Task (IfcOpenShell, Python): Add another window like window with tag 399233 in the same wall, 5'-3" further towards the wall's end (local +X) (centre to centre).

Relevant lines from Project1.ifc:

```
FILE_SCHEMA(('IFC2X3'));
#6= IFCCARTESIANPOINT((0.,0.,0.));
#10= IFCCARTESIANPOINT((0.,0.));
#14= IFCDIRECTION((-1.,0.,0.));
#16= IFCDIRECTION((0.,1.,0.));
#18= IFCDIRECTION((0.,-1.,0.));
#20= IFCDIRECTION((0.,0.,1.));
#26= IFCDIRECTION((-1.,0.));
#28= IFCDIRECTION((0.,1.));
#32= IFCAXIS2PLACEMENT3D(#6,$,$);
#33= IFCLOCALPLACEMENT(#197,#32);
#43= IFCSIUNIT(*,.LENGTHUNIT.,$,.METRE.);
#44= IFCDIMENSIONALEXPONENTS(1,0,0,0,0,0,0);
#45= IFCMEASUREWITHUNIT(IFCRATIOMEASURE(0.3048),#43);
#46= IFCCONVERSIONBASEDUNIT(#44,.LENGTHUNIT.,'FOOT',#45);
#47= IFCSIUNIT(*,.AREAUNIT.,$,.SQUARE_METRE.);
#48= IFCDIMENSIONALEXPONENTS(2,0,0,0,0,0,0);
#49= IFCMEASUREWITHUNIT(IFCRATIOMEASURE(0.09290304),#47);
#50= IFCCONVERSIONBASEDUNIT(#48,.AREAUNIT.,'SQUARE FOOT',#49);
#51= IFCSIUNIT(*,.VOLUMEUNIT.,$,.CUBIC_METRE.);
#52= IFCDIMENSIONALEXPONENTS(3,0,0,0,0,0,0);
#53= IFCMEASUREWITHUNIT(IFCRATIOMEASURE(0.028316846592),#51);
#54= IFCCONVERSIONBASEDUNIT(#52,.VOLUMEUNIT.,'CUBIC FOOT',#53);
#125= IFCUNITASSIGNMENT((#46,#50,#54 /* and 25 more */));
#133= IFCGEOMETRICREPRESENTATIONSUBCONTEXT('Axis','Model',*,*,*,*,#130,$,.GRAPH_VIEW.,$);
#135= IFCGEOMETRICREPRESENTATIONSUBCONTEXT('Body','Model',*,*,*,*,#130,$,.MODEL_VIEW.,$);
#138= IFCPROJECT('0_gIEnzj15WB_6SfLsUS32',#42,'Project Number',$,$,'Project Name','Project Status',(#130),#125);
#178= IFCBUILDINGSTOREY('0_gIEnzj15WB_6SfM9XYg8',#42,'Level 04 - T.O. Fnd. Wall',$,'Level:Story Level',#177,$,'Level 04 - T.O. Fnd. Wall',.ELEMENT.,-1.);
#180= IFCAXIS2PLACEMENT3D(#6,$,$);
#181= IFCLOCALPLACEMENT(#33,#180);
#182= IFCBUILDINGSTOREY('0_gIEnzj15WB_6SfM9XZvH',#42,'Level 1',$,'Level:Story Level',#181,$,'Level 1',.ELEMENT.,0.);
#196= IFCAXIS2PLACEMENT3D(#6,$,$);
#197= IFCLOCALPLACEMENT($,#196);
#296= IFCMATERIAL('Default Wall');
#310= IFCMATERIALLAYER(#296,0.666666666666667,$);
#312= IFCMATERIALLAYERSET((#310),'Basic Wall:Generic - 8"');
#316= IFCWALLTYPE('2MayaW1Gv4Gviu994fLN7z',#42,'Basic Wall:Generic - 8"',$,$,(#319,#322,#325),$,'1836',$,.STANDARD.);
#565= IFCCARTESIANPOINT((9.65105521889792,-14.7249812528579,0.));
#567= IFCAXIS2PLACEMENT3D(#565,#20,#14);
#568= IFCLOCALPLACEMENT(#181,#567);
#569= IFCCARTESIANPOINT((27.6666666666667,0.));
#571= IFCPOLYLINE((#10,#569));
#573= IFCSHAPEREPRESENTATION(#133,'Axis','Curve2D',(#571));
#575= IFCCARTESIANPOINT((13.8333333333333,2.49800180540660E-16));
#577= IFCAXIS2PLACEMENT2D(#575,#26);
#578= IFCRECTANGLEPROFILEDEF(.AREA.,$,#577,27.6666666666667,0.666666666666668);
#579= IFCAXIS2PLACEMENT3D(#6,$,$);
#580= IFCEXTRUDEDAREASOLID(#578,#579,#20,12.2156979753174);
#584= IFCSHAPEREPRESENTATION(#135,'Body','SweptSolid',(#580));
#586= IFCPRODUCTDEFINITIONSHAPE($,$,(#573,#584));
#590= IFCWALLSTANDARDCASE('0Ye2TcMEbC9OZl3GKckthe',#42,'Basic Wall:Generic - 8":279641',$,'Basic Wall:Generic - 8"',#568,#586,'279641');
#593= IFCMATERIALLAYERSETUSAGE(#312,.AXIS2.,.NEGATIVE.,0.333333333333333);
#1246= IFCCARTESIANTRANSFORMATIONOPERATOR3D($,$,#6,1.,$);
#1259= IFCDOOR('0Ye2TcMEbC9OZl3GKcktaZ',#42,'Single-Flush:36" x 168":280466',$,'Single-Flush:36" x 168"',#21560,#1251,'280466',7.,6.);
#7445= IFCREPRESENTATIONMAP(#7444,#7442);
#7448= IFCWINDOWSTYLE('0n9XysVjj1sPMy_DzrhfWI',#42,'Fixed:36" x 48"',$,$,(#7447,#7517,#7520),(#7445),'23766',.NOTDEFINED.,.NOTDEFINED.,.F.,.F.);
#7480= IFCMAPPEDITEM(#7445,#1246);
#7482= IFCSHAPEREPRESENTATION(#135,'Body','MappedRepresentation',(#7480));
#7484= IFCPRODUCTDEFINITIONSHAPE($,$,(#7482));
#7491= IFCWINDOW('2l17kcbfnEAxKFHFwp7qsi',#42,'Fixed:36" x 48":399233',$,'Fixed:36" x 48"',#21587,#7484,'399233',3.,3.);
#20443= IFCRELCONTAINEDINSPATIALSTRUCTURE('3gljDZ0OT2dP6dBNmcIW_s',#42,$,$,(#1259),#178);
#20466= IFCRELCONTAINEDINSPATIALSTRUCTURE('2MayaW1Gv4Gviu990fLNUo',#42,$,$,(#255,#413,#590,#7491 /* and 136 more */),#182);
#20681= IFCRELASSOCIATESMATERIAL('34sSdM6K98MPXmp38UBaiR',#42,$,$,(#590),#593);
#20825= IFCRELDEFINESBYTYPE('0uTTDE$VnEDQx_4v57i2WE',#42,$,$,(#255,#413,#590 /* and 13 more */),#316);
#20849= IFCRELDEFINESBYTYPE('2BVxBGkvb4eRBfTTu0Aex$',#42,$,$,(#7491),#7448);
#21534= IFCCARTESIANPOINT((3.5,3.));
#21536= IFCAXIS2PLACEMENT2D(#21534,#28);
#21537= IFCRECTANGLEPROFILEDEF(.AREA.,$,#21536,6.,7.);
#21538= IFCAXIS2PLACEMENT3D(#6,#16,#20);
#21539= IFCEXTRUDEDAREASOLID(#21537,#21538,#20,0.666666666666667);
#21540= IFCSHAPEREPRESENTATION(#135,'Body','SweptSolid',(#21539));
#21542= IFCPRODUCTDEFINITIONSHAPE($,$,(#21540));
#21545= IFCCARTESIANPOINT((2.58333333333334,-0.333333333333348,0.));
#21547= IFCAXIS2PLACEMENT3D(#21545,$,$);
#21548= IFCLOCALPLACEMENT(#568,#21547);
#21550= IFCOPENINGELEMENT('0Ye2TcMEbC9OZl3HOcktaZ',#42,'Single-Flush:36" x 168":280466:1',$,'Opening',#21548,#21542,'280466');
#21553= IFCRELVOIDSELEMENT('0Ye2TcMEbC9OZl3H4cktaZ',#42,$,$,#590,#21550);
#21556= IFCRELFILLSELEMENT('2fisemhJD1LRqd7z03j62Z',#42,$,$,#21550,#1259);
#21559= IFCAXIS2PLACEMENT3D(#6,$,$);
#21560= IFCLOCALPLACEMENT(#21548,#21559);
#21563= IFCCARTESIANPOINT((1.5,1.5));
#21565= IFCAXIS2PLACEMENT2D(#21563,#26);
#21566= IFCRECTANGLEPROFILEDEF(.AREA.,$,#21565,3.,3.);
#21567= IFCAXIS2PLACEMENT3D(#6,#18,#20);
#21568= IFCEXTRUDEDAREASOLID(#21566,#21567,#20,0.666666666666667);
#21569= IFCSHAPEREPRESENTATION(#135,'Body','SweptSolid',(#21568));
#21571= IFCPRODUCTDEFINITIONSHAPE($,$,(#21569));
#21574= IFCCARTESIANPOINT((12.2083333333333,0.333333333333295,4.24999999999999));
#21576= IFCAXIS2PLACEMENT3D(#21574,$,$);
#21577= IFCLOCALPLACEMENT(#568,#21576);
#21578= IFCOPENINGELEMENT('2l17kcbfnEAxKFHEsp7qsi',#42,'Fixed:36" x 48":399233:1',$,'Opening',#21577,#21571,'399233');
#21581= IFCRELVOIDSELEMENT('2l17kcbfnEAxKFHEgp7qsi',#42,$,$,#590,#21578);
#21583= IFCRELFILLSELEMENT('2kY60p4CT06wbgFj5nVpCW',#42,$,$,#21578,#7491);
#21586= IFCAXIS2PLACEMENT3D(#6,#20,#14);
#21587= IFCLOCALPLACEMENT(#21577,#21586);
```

```python
import ifcopenshell
import ifcopenshell.api.feature
import ifcopenshell.api.geometry
import ifcopenshell.api.root
import ifcopenshell.geom
import ifcopenshell.util.element
import ifcopenshell.util.placement
import ifcopenshell.util.shape
import ifcopenshell.util.unit

model = ifcopenshell.open("Project1.ifc")
unit_scale = ifcopenshell.util.unit.calculate_unit_scale(model)
settings = ifcopenshell.geom.settings()


def volume(element):
    """Net volume in cubic metres, openings subtracted."""
    shape = ifcopenshell.geom.create_shape(settings, element)
    return ifcopenshell.util.shape.get_volume(shape.geometry)


def reuse_history(source, copy):
    """copy_class also copies each property set's owner history, people and application; keep the originals."""
    for rel in copy.IsDefinedBy:
        if rel.is_a("IfcRelDefinesByProperties") and (history := rel.RelatingPropertyDefinition.OwnerHistory):
            rel.RelatingPropertyDefinition.OwnerHistory = source.OwnerHistory
            ifcopenshell.util.element.remove_deep2(model, history)


window = model.by_guid("2l17kcbfnEAxKFHFwp7qsi")
opening = window.FillsVoids[0].RelatingOpeningElement
wall = opening.VoidsElements[0].RelatingBuildingElement
before = volume(wall)
shift = ifcopenshell.util.placement.get_local_placement(wall.ObjectPlacement)[:3, 0] * 63 * 0.0254 / unit_scale

# copy_class copies the void relationship, type, container and properties, but no geometry.
new_opening = ifcopenshell.api.root.copy_class(model, product=opening)
new_opening.Representation = ifcopenshell.util.element.copy_deep(
    model, opening.Representation, exclude=["IfcGeometricRepresentationContext", "IfcRepresentationMap"]
)
new_opening.Name = 'Fixed:36" x 48"'
new_opening.Tag = None
new_window = ifcopenshell.api.root.copy_class(model, product=window)
new_window.Representation = ifcopenshell.util.element.copy_deep(
    model, window.Representation, exclude=["IfcGeometricRepresentationContext", "IfcRepresentationMap"]
)
new_window.Name = 'Fixed:36" x 48"'
new_window.Tag = None
reuse_history(window, new_window)
fills = ifcopenshell.api.feature.add_filling(model, opening=new_opening, element=new_window)
fills.OwnerHistory = new_window.OwnerHistory  # required in IFC2X3

for old, new in ((opening, new_opening), (window, new_window)):
    matrix = ifcopenshell.util.placement.get_local_placement(old.ObjectPlacement)
    matrix[:3, 3] += shift
    ifcopenshell.api.geometry.edit_object_placement(model, product=new, matrix=matrix, is_si=False)

after = volume(wall)

print(f"wall volume {before:.3f} -> {after:.3f} m3")

model.write("Project1_rev.ifc")
```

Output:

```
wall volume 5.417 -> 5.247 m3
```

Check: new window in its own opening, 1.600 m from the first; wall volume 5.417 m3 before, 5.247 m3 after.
